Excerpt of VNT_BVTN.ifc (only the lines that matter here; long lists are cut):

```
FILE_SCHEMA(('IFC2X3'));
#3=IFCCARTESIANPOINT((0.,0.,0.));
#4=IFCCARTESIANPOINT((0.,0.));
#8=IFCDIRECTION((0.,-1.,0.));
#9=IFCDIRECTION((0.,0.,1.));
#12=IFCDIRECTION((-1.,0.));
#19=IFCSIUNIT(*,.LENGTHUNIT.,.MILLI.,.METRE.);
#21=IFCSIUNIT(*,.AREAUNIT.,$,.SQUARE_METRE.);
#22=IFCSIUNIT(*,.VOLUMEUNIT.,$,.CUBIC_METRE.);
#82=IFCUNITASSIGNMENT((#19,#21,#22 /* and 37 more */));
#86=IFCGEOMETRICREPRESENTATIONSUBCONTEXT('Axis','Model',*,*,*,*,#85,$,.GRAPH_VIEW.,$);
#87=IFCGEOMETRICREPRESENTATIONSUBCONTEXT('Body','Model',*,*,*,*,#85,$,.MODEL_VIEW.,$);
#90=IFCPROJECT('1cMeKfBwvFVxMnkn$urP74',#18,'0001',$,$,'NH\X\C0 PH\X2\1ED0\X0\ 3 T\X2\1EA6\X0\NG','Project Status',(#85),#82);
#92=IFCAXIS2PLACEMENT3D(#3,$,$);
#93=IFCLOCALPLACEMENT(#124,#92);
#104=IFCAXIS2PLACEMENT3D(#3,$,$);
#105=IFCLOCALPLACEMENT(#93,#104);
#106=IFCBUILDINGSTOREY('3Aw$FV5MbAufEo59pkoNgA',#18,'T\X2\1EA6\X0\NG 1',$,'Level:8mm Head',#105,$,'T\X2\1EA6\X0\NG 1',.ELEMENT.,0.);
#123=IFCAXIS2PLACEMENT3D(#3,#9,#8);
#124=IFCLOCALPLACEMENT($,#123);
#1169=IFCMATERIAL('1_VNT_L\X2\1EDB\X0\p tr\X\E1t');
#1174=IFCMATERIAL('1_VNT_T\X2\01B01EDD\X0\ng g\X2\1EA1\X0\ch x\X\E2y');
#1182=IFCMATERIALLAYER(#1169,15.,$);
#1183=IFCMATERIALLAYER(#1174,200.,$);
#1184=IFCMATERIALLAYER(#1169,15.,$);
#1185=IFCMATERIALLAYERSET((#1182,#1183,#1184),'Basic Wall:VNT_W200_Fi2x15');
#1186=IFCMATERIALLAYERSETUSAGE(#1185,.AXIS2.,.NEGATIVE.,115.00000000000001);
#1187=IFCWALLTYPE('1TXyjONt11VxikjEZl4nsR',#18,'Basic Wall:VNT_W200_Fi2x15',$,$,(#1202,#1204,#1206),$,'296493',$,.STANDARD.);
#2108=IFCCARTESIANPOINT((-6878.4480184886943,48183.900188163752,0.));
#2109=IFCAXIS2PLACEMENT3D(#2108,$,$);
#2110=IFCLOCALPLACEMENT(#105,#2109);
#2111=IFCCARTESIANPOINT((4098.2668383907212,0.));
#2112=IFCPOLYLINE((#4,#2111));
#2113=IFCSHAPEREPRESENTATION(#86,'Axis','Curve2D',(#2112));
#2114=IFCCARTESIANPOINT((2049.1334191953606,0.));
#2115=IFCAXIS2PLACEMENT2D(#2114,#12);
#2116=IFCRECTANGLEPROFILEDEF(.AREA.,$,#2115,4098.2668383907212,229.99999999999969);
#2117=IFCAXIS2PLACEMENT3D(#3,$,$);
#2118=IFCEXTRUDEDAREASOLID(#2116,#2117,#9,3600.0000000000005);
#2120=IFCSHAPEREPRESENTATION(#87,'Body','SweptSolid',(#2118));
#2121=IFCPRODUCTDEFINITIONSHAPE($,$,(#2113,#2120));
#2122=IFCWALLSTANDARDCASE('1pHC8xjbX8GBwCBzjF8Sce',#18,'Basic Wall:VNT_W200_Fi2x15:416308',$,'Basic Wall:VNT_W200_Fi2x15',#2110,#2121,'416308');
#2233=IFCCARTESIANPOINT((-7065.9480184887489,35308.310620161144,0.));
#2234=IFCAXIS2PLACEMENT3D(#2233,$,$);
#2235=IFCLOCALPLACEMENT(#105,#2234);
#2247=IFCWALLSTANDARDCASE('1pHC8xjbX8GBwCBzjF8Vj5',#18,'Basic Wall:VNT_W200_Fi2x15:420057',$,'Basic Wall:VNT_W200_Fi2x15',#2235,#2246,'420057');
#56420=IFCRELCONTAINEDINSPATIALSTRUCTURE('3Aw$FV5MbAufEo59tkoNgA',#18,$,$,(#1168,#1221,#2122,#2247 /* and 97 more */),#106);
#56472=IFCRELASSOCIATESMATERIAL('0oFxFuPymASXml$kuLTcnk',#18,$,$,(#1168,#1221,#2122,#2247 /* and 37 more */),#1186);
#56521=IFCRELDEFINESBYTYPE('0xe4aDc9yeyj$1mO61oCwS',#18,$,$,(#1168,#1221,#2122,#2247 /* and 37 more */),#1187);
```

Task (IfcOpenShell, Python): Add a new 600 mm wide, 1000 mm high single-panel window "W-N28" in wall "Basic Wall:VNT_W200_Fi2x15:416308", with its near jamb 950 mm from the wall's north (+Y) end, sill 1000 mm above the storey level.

```python
import numpy as np
import ifcopenshell
import ifcopenshell.api.feature
import ifcopenshell.api.geometry
import ifcopenshell.api.root
import ifcopenshell.api.spatial
import ifcopenshell.api.type
import ifcopenshell.geom
import ifcopenshell.util.element
import ifcopenshell.util.placement
import ifcopenshell.util.representation
import ifcopenshell.util.shape
import ifcopenshell.util.unit

model = ifcopenshell.open("VNT_BVTN.ifc")
unit_scale = ifcopenshell.util.unit.calculate_unit_scale(model)
settings = ifcopenshell.geom.settings()


def volume(element):
    """Net volume in cubic metres, openings subtracted."""
    shape = ifcopenshell.geom.create_shape(settings, element)
    return ifcopenshell.util.shape.get_volume(shape.geometry)


wall = model.by_guid("1pHC8xjbX8GBwCBzjF8Sce")
storey = ifcopenshell.util.element.get_container(wall, ifc_class="IfcBuildingStorey")
context = ifcopenshell.util.representation.get_context(model, "Model", "Body", "MODEL_VIEW")
before = volume(wall)

width, height, from_end, sill = 0.6, 1, 0.95, 1  # metres

# The wall runs along its own X axis, and the end named is its -X end.
wall_shape = ifcopenshell.geom.create_shape(settings, wall)
x, y, z = ifcopenshell.util.shape.get_vertices(wall_shape.geometry).T
start = x.min() + from_end
face, thickness = float(y.min()), float(y.max() - y.min())
wall_matrix = ifcopenshell.util.placement.get_local_placement(wall.ObjectPlacement)
level = ifcopenshell.util.placement.get_local_placement(storey.ObjectPlacement)[2, 3]


def in_wall(x, y):
    """Placement at x, y metres in the wall's axes, at sill height."""
    matrix = wall_matrix.copy()
    matrix[:, 3] = wall_matrix @ np.array([x / unit_scale, y / unit_scale, 0.0, 1.0])
    matrix[2, 3] = level + sill / unit_scale
    return matrix


# Opening: a box that overshoots both wall faces by 50 mm.
opening = ifcopenshell.api.root.create_entity(model, ifc_class="IfcOpeningElement")
box = ifcopenshell.api.geometry.add_wall_representation(
    model, context=context, length=width, height=height, thickness=thickness + 0.1
)
ifcopenshell.api.geometry.assign_representation(model, product=opening, representation=box)
ifcopenshell.api.geometry.edit_object_placement(model, product=opening, matrix=in_wall(start, face - 0.05), is_si=False)
ifcopenshell.api.feature.add_feature(model, feature=opening, element=wall)

window = ifcopenshell.api.root.create_entity(model, ifc_class="IfcWindow", name="W-N28")
window.OverallWidth, window.OverallHeight = width / unit_scale, height / unit_scale
body = ifcopenshell.api.geometry.add_window_representation(
    model,
    context=context,
    overall_width=window.OverallWidth,
    overall_height=window.OverallHeight,
    partition_type="SINGLE_PANEL",
)
ifcopenshell.api.geometry.assign_representation(model, product=window, representation=body)
ifcopenshell.api.spatial.assign_container(model, products=[window], relating_structure=storey)
fills = ifcopenshell.api.feature.add_filling(model, opening=opening, element=window)
fills.OwnerHistory = window.OwnerHistory  # required in IFC2X3

# IFC2X3 keeps the operation on the window style.
style = ifcopenshell.api.root.create_entity(model, ifc_class="IfcWindowStyle", name="W-N28")
style.OperationType, style.ConstructionType = "SINGLE_PANEL", "NOTDEFINED"
style.ParameterTakesPrecedence = style.Sizeable = False
ifcopenshell.api.type.assign_type(model, related_objects=[window], relating_type=style)

# Centre the window in the wall's thickness.
ifcopenshell.api.geometry.edit_object_placement(model, product=window, matrix=in_wall(start, face), is_si=False)
window_shape = ifcopenshell.geom.create_shape(settings, window)
depth = ifcopenshell.util.shape.get_vertices(window_shape.geometry)[:, 1]
offset = face + thickness / 2 - (depth.min() + depth.max()) / 2
ifcopenshell.api.geometry.edit_object_placement(model, product=window, matrix=in_wall(start, offset), is_si=False)

after = volume(wall)

print(f"wall volume {before:.3f} -> {after:.3f} m3")

model.write("VNT_BVTN_edited.ifc")
```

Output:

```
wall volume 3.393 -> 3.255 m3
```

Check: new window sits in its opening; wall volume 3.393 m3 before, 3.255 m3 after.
